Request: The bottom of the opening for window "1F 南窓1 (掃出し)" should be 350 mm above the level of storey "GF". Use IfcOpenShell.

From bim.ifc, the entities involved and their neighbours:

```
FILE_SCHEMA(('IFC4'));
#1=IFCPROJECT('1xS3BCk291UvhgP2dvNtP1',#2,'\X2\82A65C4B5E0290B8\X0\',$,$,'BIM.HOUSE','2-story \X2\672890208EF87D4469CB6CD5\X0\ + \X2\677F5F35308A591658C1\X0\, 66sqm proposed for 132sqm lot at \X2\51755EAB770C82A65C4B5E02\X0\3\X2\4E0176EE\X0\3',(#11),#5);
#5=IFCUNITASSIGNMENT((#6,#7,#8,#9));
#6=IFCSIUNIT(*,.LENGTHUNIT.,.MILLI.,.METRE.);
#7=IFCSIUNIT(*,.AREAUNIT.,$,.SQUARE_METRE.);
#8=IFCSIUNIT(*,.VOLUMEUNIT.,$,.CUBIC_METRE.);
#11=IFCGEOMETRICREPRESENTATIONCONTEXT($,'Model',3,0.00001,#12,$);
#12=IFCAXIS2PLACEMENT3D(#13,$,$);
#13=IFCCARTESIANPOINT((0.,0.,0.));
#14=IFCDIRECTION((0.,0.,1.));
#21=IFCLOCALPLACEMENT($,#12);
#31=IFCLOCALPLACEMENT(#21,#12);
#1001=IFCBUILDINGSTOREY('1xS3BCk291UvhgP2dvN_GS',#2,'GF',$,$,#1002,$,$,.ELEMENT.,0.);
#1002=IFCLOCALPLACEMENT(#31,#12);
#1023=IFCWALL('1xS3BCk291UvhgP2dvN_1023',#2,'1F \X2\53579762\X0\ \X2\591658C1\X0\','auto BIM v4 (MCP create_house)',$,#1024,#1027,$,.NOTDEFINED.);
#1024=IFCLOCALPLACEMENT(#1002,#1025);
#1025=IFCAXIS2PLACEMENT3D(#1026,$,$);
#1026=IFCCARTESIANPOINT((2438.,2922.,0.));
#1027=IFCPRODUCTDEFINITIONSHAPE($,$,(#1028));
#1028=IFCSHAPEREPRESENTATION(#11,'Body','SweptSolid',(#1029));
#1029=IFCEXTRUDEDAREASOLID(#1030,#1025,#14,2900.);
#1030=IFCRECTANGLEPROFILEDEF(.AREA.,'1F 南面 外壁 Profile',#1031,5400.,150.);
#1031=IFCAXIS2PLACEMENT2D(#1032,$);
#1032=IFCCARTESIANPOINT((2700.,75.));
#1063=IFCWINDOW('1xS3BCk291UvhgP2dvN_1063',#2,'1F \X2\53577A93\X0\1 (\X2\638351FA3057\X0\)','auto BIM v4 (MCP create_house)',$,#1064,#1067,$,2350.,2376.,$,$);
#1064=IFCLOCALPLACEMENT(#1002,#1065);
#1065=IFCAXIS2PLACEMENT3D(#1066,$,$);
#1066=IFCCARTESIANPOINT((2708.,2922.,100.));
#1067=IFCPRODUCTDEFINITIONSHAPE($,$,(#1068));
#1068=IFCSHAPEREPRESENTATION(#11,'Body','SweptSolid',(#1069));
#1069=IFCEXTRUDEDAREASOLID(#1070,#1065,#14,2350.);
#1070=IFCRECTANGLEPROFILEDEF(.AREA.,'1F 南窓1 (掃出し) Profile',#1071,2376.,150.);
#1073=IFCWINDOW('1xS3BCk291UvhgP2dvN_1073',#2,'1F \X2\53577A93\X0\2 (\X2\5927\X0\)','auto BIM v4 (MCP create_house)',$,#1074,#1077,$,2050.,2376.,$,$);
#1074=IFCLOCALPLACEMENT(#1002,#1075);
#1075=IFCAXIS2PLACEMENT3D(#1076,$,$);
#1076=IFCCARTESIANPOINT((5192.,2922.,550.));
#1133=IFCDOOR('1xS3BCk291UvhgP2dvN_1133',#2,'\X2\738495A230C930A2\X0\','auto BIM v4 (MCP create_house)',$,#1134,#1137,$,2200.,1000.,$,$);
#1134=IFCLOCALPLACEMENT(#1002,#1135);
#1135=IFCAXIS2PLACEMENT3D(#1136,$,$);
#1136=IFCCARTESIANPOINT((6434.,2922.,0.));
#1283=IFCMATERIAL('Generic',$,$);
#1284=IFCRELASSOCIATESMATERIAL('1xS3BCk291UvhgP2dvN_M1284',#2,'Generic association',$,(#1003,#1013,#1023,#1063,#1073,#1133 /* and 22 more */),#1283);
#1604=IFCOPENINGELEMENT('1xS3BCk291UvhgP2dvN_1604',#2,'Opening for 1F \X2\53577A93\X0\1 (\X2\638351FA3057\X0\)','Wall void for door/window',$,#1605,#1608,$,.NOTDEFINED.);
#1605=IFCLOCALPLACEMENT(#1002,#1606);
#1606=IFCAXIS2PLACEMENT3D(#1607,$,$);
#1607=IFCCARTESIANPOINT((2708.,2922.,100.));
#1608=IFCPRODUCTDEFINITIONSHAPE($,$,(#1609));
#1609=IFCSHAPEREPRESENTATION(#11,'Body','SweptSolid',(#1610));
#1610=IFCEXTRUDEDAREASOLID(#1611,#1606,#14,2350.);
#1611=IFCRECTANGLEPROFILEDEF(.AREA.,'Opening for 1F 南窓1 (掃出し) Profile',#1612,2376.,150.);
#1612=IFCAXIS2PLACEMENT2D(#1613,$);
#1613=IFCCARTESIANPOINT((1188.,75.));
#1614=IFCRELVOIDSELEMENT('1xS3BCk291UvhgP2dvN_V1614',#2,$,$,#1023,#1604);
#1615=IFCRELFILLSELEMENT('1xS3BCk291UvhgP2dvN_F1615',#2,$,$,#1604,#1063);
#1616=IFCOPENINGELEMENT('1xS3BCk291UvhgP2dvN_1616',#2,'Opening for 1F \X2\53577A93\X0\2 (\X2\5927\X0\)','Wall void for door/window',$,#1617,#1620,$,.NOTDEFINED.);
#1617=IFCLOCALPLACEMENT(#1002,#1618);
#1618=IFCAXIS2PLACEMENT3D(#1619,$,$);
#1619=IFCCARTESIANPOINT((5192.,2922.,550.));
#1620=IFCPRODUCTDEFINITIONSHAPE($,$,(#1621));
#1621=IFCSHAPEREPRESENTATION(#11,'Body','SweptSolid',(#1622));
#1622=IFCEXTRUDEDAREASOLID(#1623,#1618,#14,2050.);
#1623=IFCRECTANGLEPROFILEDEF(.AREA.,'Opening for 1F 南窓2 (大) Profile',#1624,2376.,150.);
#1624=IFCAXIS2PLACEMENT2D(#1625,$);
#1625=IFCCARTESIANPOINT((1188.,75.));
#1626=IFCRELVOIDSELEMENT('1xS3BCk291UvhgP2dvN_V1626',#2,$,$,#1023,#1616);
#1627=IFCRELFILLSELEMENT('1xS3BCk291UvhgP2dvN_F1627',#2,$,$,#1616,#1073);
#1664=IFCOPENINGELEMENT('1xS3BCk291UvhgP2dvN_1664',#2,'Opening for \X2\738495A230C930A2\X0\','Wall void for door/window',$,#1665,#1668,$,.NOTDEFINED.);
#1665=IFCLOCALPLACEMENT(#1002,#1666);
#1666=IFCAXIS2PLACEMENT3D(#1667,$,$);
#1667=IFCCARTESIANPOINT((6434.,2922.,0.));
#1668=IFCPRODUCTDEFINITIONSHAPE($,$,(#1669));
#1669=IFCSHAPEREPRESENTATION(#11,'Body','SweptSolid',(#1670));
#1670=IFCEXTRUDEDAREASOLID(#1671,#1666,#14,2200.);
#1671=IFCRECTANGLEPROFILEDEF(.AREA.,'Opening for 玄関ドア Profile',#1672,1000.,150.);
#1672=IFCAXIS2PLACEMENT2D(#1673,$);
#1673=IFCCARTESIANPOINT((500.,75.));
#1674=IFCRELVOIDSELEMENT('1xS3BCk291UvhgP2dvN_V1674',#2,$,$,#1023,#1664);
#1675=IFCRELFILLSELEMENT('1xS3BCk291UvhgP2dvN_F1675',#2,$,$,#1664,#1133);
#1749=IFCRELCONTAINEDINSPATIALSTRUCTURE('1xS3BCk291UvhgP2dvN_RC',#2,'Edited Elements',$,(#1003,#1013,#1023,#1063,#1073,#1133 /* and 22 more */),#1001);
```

```python
import numpy as np
import ifcopenshell
import ifcopenshell.api.geometry
import ifcopenshell.geom
import ifcopenshell.util.element
import ifcopenshell.util.placement
import ifcopenshell.util.shape
import ifcopenshell.util.unit

model = ifcopenshell.open("bim.ifc")
unit_scale = ifcopenshell.util.unit.calculate_unit_scale(model)

window = model.by_guid("1xS3BCk291UvhgP2dvN_1063")
opening = window.FillsVoids[0].RelatingOpeningElement
storey = ifcopenshell.util.element.get_container(window, ifc_class="IfcBuildingStorey")
level = ifcopenshell.util.placement.get_local_placement(storey.ObjectPlacement)[2, 3]

# The opening's origin need not be at the sill, so measure its lowest point.
shape = ifcopenshell.geom.create_shape(ifcopenshell.geom.settings(), opening)
bottom = ifcopenshell.util.shape.get_shape_bottom_elevation(shape, shape.geometry) / unit_scale
dz = level + 0.35 / unit_scale - bottom

shift = np.array([0.0, 0.0, dz])
# The window is not placed relative to its opening, so move both.
for product in (opening, window):
    matrix = ifcopenshell.util.placement.get_local_placement(product.ObjectPlacement)
    matrix[:3, 3] += shift
    ifcopenshell.api.geometry.edit_object_placement(model, product=product, matrix=matrix, is_si=False)

print(f"moved by {dz * unit_scale:+.3f} m")

model.write("bim_edited.ifc")
```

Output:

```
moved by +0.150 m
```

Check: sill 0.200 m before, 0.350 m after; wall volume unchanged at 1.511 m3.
